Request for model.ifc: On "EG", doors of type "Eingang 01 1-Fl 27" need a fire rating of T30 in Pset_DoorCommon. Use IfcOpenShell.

First a look at what the model holds.

```python
import ifcopenshell
import ifcopenshell.util.element

model = ifcopenshell.open("model.ifc")
print(model.schema)
storey = next(s for s in model.by_type("IfcBuildingStorey") if s.Name == "EG")
doors = [e for e in ifcopenshell.util.element.get_decomposition(storey) if e.is_a("IfcDoor")]
seen = {}
for e in doors:
    element_type = ifcopenshell.util.element.get_type(e)
    key = (element_type.Name if element_type != e and element_type else None, ifcopenshell.util.element.get_pset(e, "Pset_DoorCommon", "FireRating"))
    seen[key] = seen.get(key, 0) + 1
for (name, value), count in sorted(seen.items(), key=str):
    print(count, "x", name, "|", value)
```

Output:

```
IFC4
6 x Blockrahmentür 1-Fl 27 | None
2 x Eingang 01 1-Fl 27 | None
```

```python
import ifcopenshell
import ifcopenshell.api.pset
import ifcopenshell.util.element

model = ifcopenshell.open("model.ifc")

storey = next(s for s in model.by_type("IfcBuildingStorey") if s.Name == "EG")
doors = [e for e in ifcopenshell.util.element.get_decomposition(storey) if e.is_a("IfcDoor")]

count = 0
for e in doors:
    element_type = ifcopenshell.util.element.get_type(e)
    if element_type in (None, e) or element_type.Name != "Eingang 01 1-Fl 27":
        continue
    # add_pset returns the element's existing set when there is one.
    pset = ifcopenshell.api.pset.add_pset(model, product=e, name="Pset_DoorCommon")
    ifcopenshell.api.pset.edit_pset(model, pset=pset, properties={"FireRating": "T30"})
    count += 1

print(count, "doors updated")

model.write("model_updated.ifc")
```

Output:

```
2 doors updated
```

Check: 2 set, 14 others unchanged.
